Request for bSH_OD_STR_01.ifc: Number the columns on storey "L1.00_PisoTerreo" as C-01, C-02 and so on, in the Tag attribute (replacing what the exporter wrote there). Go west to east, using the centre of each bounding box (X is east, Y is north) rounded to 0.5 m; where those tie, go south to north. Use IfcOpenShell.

First a look at what the model holds.

```python
import ifcopenshell
import ifcopenshell.util.element
import ifcopenshell.util.placement

model = ifcopenshell.open("bSH_OD_STR_01.ifc")
print(model.schema)
storey = next(s for s in model.by_type("IfcBuildingStorey") if s.Name == "L1.00_PisoTerreo")
columns = [e for e in ifcopenshell.util.element.get_decomposition(storey) if e.is_a("IfcColumn")]
for e in sorted(columns, key=lambda e: e.id()):
    origin = ifcopenshell.util.placement.get_local_placement(e.ObjectPlacement)[:3, 3]
    print(e.id(), e.Tag, e.Name, origin.round(2) + 0.0, sep=" | ")
```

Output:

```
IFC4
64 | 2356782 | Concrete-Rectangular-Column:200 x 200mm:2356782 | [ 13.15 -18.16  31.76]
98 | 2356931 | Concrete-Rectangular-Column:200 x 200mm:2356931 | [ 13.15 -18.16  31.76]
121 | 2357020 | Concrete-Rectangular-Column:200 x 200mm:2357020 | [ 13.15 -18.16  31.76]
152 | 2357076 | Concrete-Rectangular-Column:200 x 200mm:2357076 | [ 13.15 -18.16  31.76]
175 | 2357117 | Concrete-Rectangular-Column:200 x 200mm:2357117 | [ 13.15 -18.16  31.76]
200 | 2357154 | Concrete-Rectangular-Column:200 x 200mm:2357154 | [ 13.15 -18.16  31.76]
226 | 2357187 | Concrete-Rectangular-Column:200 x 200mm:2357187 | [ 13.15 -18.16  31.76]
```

```python
import ifcopenshell
import ifcopenshell.geom
import ifcopenshell.util.element
import ifcopenshell.util.shape

model = ifcopenshell.open("bSH_OD_STR_01.ifc")
settings = ifcopenshell.geom.settings()
settings.set("use-world-coords", True)


def centre(element):
    shape = ifcopenshell.geom.create_shape(settings, element)
    return ifcopenshell.util.shape.get_bbox_centroid(shape.geometry)


storey = next(s for s in model.by_type("IfcBuildingStorey") if s.Name == "L1.00_PisoTerreo")
columns = [e for e in ifcopenshell.util.element.get_decomposition(storey) if e.is_a("IfcColumn")]

# Insertion points can sit at a corner or the storey origin, so sort by the geometry (in metres).
centres = {e: centre(e) for e in columns}
columns.sort(key=lambda e: (round(centres[e][0] / 0.5), centres[e][1]))

for i, e in enumerate(columns, start=1):
    number = f"C-{i:02d}"
    e.Tag = number
    print(e.id(), number)

model.write("bSH_OD_STR_01-out.ifc")
```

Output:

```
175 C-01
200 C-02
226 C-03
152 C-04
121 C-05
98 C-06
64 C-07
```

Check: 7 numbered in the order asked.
